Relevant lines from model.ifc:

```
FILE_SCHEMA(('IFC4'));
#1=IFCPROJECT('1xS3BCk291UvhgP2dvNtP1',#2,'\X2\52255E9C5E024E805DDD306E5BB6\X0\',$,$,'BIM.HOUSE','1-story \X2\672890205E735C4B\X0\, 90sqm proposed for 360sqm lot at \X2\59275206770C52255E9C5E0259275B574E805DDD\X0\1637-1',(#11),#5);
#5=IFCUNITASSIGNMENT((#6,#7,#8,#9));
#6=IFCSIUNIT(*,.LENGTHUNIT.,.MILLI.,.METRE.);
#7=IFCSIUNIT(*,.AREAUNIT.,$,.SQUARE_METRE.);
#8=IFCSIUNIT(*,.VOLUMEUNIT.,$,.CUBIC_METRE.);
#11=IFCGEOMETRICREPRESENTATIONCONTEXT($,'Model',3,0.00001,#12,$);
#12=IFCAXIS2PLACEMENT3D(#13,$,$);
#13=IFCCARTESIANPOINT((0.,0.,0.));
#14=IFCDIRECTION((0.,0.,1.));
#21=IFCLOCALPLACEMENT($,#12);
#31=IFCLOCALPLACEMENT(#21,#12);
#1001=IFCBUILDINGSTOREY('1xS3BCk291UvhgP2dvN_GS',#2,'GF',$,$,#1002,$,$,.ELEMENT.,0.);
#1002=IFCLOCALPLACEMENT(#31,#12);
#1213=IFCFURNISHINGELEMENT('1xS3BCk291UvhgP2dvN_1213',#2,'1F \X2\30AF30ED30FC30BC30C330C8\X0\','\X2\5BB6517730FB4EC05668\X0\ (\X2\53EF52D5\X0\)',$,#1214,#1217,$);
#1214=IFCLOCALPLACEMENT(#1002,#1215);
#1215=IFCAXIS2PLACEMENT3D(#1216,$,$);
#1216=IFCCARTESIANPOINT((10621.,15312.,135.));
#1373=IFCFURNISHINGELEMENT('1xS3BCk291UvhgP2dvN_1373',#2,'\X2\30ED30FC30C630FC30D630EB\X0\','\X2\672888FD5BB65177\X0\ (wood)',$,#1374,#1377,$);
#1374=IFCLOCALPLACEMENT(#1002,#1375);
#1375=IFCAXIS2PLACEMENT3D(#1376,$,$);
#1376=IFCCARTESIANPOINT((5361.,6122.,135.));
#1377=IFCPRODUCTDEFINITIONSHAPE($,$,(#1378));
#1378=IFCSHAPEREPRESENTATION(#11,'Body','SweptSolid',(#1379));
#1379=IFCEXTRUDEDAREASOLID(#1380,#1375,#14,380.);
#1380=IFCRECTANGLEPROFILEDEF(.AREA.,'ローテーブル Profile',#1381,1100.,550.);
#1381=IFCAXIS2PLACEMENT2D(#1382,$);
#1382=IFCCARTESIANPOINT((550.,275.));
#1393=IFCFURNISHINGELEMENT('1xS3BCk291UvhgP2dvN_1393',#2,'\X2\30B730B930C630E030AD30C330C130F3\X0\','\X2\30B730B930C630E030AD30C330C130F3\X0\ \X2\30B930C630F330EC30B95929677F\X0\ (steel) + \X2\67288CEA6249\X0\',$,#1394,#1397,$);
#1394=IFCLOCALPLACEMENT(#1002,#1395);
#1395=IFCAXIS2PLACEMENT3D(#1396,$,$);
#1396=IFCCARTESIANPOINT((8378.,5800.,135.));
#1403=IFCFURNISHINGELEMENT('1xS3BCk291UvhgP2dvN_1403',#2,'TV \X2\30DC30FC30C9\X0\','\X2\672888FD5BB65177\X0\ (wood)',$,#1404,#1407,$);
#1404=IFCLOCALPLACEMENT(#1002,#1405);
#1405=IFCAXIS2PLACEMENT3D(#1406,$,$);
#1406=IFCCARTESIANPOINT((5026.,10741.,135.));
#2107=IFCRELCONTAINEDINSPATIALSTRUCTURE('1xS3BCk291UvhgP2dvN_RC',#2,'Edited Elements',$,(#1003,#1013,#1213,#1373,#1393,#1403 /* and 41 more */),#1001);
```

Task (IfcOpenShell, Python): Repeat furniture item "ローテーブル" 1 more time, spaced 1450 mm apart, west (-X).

```python
import numpy as np
import ifcopenshell
import ifcopenshell.api.geometry
import ifcopenshell.api.root
import ifcopenshell.util.element
import ifcopenshell.util.placement
import ifcopenshell.util.unit

model = ifcopenshell.open("model.ifc")
unit_scale = ifcopenshell.util.unit.calculate_unit_scale(model)


def reuse_history(source, copy):
    """copy_class also copies each property set's owner history, people and application; keep the originals."""
    for rel in copy.IsDefinedBy:
        if rel.is_a("IfcRelDefinesByProperties") and (history := rel.RelatingPropertyDefinition.OwnerHistory):
            rel.RelatingPropertyDefinition.OwnerHistory = source.OwnerHistory
            ifcopenshell.util.element.remove_deep2(model, history)


source = model.by_guid("1xS3BCk291UvhgP2dvN_1373")
base = ifcopenshell.util.placement.get_local_placement(source.ObjectPlacement)
step = np.array([-1.0, 0.0, 0.0]) * 1.45 / unit_scale

for i in range(1, 2):
    copy = ifcopenshell.api.root.copy_class(model, product=source)
    copy.Representation = ifcopenshell.util.element.copy_deep(
        model, source.Representation, exclude=["IfcGeometricRepresentationContext", "IfcRepresentationMap"]
    )
    reuse_history(source, copy)
    matrix = base.copy()
    matrix[:3, 3] += i * step
    print("added at", matrix[:3, 3].round(3) + 0.0)
    ifcopenshell.api.geometry.edit_object_placement(model, product=copy, matrix=matrix, is_si=False)

model.write("model-out.ifc")
```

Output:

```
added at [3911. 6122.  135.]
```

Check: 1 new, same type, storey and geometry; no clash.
